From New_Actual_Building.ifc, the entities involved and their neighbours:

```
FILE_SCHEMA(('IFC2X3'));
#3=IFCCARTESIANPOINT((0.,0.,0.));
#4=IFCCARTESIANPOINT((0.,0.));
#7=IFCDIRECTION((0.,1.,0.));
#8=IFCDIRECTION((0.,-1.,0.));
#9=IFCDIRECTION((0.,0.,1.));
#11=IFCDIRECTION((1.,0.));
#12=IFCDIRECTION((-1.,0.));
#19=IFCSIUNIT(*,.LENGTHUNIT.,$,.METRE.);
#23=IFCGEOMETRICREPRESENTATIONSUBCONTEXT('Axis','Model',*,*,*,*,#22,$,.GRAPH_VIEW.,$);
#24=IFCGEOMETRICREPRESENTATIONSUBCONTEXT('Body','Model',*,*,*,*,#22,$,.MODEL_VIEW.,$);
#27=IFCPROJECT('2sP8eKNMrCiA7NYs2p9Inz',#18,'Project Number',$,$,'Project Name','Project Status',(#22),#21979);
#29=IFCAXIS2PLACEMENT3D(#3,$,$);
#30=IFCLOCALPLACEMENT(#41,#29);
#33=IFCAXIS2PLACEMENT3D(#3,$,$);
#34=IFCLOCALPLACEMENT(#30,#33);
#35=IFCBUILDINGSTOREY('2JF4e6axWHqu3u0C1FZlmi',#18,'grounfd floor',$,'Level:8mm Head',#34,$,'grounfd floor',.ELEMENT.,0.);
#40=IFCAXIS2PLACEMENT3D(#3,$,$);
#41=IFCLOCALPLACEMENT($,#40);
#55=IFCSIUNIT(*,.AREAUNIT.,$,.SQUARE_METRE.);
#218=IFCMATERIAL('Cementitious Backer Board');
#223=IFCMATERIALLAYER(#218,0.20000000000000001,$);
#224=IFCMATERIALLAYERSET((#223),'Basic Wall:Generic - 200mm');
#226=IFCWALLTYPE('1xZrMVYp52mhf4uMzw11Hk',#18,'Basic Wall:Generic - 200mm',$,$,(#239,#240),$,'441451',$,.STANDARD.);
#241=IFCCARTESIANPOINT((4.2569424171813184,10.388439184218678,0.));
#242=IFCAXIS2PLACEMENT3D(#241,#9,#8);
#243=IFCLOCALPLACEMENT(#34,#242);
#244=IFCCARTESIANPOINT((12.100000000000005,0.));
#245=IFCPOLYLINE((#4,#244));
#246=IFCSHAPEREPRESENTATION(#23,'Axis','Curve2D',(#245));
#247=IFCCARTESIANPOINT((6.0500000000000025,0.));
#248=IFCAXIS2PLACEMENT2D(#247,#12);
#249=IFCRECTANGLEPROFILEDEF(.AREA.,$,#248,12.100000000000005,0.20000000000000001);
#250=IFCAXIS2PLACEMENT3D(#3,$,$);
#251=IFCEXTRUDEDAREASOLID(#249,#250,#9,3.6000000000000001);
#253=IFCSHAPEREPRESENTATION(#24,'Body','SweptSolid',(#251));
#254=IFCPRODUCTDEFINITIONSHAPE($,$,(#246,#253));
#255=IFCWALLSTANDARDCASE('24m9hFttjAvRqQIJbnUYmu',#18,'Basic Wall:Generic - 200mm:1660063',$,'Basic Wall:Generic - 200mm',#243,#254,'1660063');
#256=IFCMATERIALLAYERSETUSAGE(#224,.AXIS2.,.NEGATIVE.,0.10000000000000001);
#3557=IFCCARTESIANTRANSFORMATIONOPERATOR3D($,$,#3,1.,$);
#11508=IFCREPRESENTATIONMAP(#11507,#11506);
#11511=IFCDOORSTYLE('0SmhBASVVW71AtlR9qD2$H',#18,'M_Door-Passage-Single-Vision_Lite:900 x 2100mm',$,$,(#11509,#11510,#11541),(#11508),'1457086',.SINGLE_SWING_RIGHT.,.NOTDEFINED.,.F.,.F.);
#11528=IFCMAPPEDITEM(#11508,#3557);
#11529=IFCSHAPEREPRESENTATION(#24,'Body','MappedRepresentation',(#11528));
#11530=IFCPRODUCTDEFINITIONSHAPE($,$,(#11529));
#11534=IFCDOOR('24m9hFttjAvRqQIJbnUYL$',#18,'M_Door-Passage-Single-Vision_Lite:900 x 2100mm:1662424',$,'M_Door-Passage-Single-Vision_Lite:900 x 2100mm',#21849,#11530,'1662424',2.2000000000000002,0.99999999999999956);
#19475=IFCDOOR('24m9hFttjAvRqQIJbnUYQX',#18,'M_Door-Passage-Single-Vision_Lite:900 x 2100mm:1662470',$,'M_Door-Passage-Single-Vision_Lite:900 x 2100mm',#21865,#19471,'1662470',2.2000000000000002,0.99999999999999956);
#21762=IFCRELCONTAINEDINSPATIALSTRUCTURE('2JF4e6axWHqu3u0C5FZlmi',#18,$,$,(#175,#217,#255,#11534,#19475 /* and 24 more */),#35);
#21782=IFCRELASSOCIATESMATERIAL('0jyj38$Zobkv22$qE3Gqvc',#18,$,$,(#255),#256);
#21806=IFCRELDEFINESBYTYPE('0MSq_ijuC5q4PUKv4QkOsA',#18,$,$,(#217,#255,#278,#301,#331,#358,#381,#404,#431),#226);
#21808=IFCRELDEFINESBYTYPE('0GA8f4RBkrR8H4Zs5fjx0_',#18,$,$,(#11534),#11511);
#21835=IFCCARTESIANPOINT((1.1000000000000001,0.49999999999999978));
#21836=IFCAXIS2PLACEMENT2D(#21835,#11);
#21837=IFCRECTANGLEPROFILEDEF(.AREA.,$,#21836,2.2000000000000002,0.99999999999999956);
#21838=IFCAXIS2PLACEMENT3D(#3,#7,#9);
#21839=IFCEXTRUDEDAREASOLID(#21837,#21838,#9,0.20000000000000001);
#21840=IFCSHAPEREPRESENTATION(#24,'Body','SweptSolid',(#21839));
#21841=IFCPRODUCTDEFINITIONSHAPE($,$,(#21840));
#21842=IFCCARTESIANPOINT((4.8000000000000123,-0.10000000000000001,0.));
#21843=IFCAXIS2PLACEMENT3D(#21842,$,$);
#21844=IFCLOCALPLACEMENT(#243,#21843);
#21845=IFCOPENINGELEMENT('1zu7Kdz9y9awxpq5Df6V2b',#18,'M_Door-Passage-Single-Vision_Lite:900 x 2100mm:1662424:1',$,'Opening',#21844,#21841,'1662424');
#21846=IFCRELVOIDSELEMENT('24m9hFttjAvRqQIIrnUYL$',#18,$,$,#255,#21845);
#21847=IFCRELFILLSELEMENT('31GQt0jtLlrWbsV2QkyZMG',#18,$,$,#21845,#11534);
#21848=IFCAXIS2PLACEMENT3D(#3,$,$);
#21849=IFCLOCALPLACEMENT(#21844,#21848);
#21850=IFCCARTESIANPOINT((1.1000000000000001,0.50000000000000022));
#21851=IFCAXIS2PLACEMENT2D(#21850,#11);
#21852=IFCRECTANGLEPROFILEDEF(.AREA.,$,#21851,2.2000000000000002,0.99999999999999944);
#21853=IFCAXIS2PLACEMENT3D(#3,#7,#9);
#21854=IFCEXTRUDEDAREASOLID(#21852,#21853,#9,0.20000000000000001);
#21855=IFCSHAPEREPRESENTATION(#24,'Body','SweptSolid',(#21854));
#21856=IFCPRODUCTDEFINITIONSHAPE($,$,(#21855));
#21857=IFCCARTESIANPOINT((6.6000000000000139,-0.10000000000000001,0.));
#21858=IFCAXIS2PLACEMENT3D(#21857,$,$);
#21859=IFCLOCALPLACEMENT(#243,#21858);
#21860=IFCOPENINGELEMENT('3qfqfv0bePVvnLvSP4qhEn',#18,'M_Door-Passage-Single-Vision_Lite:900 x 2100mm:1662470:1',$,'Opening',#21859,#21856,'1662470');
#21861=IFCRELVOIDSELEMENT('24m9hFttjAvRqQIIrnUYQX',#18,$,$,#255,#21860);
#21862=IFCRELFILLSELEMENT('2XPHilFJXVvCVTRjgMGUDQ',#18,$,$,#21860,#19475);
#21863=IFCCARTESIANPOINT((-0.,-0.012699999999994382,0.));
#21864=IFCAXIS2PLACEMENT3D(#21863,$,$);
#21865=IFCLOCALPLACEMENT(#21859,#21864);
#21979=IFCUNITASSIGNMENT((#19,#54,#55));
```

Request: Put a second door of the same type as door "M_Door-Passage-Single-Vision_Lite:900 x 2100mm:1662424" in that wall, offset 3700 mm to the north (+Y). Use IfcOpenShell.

```python
import ifcopenshell
import ifcopenshell.api.feature
import ifcopenshell.api.geometry
import ifcopenshell.api.root
import ifcopenshell.geom
import ifcopenshell.util.element
import ifcopenshell.util.placement
import ifcopenshell.util.shape

model = ifcopenshell.open("New_Actual_Building.ifc")
settings = ifcopenshell.geom.settings()


def volume(element):
    """Net volume in cubic metres, openings subtracted."""
    shape = ifcopenshell.geom.create_shape(settings, element)
    return ifcopenshell.util.shape.get_volume(shape.geometry)


def reuse_history(source, copy):
    """copy_class also copies each property set's owner history, people and application; keep the originals."""
    for rel in copy.IsDefinedBy:
        if rel.is_a("IfcRelDefinesByProperties") and (history := rel.RelatingPropertyDefinition.OwnerHistory):
            rel.RelatingPropertyDefinition.OwnerHistory = source.OwnerHistory
            ifcopenshell.util.element.remove_deep2(model, history)


door = model.by_id(11534)
opening = door.FillsVoids[0].RelatingOpeningElement
wall = opening.VoidsElements[0].RelatingBuildingElement
before = volume(wall)
shift = ifcopenshell.util.placement.get_local_placement(wall.ObjectPlacement)[:3, 0] * -3.7

# copy_class copies the void relationship, type, container and properties, but no geometry.
new_opening = ifcopenshell.api.root.copy_class(model, product=opening)
new_opening.Representation = ifcopenshell.util.element.copy_deep(
    model, opening.Representation, exclude=["IfcGeometricRepresentationContext", "IfcRepresentationMap"]
)
new_opening.Name = "M_Door-Passage-Single-Vision_Lite:900 x 2100mm"
new_opening.Tag = None
new_door = ifcopenshell.api.root.copy_class(model, product=door)
new_door.Representation = ifcopenshell.util.element.copy_deep(
    model, door.Representation, exclude=["IfcGeometricRepresentationContext", "IfcRepresentationMap"]
)
new_door.Name = "M_Door-Passage-Single-Vision_Lite:900 x 2100mm"
new_door.Tag = None
reuse_history(door, new_door)
fills = ifcopenshell.api.feature.add_filling(model, opening=new_opening, element=new_door)
fills.OwnerHistory = new_door.OwnerHistory  # required in IFC2X3

for old, new in ((opening, new_opening), (door, new_door)):
    matrix = ifcopenshell.util.placement.get_local_placement(old.ObjectPlacement)
    matrix[:3, 3] += shift
    ifcopenshell.api.geometry.edit_object_placement(model, product=new, matrix=matrix, is_si=False)

after = volume(wall)

print(f"wall volume {before:.3f} -> {after:.3f} m3")

model.write("New_Actual_Building_v2.ifc")
```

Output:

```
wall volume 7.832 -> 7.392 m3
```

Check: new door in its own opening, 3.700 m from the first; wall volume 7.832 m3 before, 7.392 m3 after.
